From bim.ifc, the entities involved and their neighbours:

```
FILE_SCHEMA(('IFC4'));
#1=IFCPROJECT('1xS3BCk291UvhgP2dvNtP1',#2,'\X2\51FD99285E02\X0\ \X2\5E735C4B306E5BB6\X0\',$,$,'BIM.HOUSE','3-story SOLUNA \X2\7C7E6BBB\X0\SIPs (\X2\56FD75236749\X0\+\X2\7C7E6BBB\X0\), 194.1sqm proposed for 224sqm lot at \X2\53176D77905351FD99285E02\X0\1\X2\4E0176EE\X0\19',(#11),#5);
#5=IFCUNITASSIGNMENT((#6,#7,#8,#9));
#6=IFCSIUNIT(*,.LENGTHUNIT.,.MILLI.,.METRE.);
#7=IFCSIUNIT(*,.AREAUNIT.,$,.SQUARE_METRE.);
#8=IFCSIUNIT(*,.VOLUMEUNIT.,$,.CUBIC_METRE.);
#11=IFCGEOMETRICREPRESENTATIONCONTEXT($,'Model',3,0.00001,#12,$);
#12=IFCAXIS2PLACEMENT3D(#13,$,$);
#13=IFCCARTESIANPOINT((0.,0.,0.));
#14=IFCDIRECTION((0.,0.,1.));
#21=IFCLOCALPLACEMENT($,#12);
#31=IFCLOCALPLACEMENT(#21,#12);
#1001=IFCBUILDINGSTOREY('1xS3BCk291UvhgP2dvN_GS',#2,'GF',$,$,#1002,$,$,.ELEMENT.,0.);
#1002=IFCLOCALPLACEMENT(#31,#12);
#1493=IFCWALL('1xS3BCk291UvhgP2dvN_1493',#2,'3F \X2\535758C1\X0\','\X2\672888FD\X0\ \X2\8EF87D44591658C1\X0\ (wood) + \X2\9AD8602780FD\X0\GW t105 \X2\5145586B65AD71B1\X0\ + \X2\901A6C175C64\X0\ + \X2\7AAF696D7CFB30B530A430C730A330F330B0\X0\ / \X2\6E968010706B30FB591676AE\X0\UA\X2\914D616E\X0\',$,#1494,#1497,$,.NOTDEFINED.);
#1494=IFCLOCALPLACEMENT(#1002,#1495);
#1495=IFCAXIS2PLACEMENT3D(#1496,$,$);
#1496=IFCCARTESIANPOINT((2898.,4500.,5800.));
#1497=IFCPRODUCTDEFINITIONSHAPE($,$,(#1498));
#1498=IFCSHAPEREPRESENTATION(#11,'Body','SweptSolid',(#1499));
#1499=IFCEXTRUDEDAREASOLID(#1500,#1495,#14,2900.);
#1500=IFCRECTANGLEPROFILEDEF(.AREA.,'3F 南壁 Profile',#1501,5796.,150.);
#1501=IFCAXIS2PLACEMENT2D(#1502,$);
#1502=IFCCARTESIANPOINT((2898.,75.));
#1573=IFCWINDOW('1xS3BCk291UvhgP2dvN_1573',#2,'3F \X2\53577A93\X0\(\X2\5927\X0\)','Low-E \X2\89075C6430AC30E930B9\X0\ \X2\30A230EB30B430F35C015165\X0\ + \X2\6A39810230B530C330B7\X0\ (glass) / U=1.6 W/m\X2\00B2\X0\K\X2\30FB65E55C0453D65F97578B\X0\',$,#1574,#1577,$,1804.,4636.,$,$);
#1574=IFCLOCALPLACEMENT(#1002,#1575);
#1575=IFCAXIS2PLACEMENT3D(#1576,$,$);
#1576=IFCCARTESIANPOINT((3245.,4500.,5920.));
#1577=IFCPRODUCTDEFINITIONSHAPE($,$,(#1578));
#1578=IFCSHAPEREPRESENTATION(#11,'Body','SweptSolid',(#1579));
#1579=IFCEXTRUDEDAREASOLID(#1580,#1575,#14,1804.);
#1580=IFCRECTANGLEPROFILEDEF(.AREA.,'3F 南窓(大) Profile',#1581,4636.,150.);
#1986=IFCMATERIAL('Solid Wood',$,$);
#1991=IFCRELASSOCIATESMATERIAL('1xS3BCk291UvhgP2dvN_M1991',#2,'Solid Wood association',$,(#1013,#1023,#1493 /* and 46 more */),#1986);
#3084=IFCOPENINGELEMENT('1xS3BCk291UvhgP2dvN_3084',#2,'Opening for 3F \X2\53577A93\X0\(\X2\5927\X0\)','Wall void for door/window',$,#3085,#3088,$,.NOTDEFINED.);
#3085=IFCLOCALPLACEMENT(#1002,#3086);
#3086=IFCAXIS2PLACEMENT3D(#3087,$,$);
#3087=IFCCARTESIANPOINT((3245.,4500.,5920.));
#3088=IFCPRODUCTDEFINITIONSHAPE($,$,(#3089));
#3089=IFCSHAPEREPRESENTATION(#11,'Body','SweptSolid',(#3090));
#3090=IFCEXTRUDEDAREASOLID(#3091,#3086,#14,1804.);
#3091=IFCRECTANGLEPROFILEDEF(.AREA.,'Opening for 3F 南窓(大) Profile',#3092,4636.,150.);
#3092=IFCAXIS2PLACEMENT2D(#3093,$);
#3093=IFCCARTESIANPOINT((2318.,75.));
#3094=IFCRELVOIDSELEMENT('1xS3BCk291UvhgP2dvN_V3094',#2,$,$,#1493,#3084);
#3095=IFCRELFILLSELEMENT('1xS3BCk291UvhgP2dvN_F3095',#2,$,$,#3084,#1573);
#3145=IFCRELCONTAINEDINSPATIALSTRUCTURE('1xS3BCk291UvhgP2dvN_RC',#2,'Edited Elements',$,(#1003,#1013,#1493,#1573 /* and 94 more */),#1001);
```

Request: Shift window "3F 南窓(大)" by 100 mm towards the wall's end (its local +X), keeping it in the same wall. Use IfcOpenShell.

```python
import ifcopenshell
import ifcopenshell.api.geometry
import ifcopenshell.util.placement
import ifcopenshell.util.unit

model = ifcopenshell.open("bim.ifc")
unit_scale = ifcopenshell.util.unit.calculate_unit_scale(model)

window = model.by_id(1573)
opening = window.FillsVoids[0].RelatingOpeningElement
wall = opening.VoidsElements[0].RelatingBuildingElement

wall_matrix = ifcopenshell.util.placement.get_local_placement(wall.ObjectPlacement)
shift = wall_matrix[:3, 0] * 0.1 / unit_scale
before = ifcopenshell.util.placement.get_local_placement(window.ObjectPlacement)[:3, 3].copy()

# The window is not placed relative to its opening, so move both.
for product in (opening, window):
    matrix = ifcopenshell.util.placement.get_local_placement(product.ObjectPlacement)
    matrix[:3, 3] += shift
    ifcopenshell.api.geometry.edit_object_placement(model, product=product, matrix=matrix, is_si=False)

after = ifcopenshell.util.placement.get_local_placement(window.ObjectPlacement)[:3, 3]
print("window moved by", (after - before).round(3) + 0.0)

model.write("bim-out.ifc")
```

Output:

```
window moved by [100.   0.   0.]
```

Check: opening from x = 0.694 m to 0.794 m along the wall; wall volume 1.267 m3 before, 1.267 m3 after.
